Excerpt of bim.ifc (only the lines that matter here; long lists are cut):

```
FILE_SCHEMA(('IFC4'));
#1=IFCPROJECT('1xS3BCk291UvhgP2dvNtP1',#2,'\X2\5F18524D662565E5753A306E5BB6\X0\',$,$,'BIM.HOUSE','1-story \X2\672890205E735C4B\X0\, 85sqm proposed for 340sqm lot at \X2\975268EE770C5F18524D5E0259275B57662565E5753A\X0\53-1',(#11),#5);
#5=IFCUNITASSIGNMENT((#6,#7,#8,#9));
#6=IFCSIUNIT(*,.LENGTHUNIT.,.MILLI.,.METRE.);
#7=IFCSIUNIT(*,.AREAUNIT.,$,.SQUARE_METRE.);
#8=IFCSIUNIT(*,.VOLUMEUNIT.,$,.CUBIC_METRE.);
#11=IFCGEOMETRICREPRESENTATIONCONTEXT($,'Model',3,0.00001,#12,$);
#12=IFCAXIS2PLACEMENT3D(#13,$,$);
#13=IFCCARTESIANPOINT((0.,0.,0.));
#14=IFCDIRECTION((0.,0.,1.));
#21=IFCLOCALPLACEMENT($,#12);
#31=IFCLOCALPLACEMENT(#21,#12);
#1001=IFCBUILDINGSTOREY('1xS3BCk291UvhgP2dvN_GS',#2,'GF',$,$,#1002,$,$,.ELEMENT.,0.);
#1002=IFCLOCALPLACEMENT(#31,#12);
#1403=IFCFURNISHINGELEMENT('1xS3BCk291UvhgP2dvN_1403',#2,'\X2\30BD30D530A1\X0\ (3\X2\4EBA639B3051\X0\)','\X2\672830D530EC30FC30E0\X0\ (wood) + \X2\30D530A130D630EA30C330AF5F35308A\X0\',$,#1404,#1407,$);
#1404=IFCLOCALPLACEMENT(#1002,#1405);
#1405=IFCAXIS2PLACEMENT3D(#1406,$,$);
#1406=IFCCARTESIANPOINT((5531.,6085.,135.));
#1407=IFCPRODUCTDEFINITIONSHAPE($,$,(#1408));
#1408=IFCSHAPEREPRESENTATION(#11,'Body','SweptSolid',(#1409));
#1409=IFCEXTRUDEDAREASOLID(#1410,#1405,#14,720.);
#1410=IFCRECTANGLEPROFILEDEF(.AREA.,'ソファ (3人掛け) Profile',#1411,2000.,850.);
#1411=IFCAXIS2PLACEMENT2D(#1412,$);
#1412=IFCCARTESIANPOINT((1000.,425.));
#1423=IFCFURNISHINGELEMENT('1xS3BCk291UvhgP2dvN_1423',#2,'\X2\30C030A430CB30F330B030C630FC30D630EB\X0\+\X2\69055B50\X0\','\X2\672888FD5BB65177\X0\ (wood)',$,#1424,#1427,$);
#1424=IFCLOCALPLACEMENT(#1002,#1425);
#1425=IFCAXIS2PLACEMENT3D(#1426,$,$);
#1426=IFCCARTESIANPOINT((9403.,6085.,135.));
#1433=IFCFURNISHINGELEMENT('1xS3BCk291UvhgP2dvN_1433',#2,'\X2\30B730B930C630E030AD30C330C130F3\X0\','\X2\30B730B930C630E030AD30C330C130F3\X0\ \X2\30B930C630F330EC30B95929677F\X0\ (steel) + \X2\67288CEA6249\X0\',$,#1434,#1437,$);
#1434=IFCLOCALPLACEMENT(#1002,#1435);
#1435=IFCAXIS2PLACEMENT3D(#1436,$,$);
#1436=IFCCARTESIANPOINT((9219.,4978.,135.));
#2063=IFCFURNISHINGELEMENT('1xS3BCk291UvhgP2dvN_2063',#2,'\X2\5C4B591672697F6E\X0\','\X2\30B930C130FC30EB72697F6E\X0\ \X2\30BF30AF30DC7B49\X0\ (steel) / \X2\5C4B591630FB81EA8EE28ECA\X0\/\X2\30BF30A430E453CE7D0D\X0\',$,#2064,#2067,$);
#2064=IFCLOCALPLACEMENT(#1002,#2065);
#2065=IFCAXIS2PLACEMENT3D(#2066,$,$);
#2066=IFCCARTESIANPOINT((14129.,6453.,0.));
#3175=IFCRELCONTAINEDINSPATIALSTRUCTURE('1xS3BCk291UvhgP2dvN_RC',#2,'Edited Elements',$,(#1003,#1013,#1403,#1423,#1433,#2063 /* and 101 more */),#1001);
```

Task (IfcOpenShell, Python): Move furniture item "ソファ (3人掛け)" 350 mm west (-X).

```python
import ifcopenshell
import ifcopenshell.api.geometry
import ifcopenshell.util.placement

model = ifcopenshell.open("bim.ifc")

item = model.by_guid("1xS3BCk291UvhgP2dvN_1403")
matrix = ifcopenshell.util.placement.get_local_placement(item.ObjectPlacement)
matrix[0, 3] -= 350.0
ifcopenshell.api.geometry.edit_object_placement(model, product=item, matrix=matrix, is_si=False)

print(ifcopenshell.util.placement.get_local_placement(item.ObjectPlacement).round(3) + 0.0)

model.write("bim_updated.ifc")
```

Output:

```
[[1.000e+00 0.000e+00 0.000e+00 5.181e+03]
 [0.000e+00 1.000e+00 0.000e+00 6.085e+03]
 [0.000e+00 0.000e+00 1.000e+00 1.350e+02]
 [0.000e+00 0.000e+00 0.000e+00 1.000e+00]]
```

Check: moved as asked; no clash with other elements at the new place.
